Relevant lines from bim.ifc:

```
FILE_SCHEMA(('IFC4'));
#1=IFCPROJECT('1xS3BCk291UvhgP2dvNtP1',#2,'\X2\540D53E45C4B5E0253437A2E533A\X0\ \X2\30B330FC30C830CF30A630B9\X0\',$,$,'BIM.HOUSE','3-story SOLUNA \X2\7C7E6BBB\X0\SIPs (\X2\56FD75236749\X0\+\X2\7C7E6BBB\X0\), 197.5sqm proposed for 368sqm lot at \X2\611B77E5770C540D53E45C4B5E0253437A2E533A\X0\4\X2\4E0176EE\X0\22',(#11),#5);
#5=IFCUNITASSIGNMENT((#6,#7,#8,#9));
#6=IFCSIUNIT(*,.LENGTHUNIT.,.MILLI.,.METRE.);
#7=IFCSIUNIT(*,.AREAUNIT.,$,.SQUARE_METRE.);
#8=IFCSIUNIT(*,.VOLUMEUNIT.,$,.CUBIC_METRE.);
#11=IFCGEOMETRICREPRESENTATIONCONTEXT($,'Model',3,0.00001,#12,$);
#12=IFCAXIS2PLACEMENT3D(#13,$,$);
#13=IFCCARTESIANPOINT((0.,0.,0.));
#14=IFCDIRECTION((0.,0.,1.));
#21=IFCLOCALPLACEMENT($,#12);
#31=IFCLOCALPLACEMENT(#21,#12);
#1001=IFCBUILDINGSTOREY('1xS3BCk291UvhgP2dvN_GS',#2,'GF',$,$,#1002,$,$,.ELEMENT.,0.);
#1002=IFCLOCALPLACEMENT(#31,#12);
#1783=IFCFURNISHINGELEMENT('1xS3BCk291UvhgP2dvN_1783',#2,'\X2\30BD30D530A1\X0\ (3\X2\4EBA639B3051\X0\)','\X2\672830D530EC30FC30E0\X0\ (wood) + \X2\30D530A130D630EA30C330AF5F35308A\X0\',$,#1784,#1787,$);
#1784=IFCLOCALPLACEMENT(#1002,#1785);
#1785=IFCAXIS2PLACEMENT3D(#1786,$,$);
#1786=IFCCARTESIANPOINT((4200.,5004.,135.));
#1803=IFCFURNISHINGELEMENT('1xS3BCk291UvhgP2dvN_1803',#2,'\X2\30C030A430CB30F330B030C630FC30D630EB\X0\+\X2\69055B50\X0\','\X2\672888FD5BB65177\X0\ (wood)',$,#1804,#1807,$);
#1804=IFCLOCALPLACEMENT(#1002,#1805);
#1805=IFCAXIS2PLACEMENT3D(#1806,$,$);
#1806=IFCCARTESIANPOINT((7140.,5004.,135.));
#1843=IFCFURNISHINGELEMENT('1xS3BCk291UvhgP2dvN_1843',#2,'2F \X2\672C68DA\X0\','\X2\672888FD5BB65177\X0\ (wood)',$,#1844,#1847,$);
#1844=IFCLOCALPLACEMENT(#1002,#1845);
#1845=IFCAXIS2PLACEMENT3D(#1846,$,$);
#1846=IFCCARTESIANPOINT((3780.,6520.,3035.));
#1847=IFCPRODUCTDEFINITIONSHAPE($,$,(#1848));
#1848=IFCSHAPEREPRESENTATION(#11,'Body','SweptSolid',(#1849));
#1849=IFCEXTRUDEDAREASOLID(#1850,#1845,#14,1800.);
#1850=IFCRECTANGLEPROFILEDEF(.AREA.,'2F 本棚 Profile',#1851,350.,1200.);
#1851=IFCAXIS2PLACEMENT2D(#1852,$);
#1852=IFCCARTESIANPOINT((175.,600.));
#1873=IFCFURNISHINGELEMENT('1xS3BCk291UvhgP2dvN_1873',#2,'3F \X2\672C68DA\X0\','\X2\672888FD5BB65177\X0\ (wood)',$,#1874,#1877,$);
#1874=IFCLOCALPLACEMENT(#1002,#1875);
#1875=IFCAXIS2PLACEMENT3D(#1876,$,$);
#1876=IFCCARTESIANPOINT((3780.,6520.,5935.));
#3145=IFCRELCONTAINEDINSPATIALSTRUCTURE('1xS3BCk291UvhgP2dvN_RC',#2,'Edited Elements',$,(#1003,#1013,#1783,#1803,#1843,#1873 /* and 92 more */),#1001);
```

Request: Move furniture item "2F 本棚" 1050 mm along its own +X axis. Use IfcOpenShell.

```python
import ifcopenshell
import ifcopenshell.api.geometry
import ifcopenshell.util.placement

model = ifcopenshell.open("bim.ifc")

item = model.by_guid("1xS3BCk291UvhgP2dvN_1843")
matrix = ifcopenshell.util.placement.get_local_placement(item.ObjectPlacement)
matrix[:3, 3] += matrix[:3, 0] * 1050.0
ifcopenshell.api.geometry.edit_object_placement(model, product=item, matrix=matrix, is_si=False)

print(ifcopenshell.util.placement.get_local_placement(item.ObjectPlacement).round(3) + 0.0)

model.write("bim_rev.ifc")
```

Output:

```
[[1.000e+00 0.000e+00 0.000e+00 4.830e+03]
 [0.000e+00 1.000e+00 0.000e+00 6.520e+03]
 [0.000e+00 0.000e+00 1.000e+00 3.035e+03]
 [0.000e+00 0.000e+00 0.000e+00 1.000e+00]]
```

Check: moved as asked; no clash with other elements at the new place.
